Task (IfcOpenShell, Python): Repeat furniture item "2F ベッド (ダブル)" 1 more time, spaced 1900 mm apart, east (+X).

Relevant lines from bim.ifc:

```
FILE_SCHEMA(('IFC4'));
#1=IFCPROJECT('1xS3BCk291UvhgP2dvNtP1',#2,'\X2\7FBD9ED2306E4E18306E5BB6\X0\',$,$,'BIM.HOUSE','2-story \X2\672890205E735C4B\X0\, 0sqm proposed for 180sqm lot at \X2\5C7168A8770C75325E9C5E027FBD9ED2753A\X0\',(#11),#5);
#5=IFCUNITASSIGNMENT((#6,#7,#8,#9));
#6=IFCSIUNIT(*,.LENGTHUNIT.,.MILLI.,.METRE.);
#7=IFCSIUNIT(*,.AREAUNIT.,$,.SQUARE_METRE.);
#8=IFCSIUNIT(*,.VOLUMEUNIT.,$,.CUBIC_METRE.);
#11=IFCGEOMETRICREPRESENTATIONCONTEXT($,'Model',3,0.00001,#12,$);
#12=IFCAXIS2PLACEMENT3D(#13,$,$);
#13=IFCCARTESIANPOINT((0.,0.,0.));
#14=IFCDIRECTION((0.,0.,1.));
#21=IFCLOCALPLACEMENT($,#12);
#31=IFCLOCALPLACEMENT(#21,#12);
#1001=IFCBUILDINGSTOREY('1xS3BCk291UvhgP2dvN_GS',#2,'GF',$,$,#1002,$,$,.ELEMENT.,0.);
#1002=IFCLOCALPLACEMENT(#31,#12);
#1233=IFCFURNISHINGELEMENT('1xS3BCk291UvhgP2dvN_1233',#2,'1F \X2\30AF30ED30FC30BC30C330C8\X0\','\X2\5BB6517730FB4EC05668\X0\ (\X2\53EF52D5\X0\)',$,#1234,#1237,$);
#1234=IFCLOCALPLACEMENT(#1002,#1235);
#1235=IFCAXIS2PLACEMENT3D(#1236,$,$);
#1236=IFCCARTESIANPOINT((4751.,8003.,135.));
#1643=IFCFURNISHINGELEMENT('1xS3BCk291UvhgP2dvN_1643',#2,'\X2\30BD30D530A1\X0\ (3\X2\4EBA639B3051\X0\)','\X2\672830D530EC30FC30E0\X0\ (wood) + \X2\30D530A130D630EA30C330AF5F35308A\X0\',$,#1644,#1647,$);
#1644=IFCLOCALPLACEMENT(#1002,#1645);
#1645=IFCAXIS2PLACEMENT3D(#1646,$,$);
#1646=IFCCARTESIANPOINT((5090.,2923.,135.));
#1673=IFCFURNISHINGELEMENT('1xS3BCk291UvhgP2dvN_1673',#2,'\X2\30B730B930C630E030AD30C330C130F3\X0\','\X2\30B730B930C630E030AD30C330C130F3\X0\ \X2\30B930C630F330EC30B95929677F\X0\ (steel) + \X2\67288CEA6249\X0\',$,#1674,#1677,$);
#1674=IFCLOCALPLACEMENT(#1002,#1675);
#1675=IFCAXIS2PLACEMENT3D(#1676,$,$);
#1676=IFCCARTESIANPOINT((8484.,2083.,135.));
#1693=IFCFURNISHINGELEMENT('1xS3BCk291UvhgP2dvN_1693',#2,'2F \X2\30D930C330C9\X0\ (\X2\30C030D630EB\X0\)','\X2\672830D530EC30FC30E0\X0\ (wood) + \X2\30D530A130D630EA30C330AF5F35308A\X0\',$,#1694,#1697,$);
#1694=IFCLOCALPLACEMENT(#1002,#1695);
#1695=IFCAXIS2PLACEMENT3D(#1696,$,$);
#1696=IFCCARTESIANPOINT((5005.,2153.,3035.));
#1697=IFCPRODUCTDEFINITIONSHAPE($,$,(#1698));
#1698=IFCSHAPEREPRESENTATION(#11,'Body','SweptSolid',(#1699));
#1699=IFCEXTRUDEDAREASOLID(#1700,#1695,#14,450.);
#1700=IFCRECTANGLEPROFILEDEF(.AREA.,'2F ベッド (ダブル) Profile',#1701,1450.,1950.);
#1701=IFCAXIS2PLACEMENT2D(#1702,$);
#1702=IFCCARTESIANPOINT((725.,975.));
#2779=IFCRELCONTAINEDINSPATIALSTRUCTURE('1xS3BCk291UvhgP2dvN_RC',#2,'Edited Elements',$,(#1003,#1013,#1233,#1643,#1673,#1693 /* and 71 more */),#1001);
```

```python
import numpy as np
import ifcopenshell
import ifcopenshell.api.geometry
import ifcopenshell.api.root
import ifcopenshell.util.element
import ifcopenshell.util.placement
import ifcopenshell.util.unit

model = ifcopenshell.open("bim.ifc")
unit_scale = ifcopenshell.util.unit.calculate_unit_scale(model)


def reuse_history(source, copy):
    """copy_class also copies each property set's owner history, people and application; keep the originals."""
    for rel in copy.IsDefinedBy:
        if rel.is_a("IfcRelDefinesByProperties") and (history := rel.RelatingPropertyDefinition.OwnerHistory):
            rel.RelatingPropertyDefinition.OwnerHistory = source.OwnerHistory
            ifcopenshell.util.element.remove_deep2(model, history)


source = model.by_id(1693)
base = ifcopenshell.util.placement.get_local_placement(source.ObjectPlacement)
step = np.array([1.0, 0.0, 0.0]) * 1.9 / unit_scale

for i in range(1, 2):
    copy = ifcopenshell.api.root.copy_class(model, product=source)
    copy.Representation = ifcopenshell.util.element.copy_deep(
        model, source.Representation, exclude=["IfcGeometricRepresentationContext", "IfcRepresentationMap"]
    )
    reuse_history(source, copy)
    matrix = base.copy()
    matrix[:3, 3] += i * step
    print("added at", matrix[:3, 3].round(3) + 0.0)
    ifcopenshell.api.geometry.edit_object_placement(model, product=copy, matrix=matrix, is_si=False)

model.write("bim_v2.ifc")
```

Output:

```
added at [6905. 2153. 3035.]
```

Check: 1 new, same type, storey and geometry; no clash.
